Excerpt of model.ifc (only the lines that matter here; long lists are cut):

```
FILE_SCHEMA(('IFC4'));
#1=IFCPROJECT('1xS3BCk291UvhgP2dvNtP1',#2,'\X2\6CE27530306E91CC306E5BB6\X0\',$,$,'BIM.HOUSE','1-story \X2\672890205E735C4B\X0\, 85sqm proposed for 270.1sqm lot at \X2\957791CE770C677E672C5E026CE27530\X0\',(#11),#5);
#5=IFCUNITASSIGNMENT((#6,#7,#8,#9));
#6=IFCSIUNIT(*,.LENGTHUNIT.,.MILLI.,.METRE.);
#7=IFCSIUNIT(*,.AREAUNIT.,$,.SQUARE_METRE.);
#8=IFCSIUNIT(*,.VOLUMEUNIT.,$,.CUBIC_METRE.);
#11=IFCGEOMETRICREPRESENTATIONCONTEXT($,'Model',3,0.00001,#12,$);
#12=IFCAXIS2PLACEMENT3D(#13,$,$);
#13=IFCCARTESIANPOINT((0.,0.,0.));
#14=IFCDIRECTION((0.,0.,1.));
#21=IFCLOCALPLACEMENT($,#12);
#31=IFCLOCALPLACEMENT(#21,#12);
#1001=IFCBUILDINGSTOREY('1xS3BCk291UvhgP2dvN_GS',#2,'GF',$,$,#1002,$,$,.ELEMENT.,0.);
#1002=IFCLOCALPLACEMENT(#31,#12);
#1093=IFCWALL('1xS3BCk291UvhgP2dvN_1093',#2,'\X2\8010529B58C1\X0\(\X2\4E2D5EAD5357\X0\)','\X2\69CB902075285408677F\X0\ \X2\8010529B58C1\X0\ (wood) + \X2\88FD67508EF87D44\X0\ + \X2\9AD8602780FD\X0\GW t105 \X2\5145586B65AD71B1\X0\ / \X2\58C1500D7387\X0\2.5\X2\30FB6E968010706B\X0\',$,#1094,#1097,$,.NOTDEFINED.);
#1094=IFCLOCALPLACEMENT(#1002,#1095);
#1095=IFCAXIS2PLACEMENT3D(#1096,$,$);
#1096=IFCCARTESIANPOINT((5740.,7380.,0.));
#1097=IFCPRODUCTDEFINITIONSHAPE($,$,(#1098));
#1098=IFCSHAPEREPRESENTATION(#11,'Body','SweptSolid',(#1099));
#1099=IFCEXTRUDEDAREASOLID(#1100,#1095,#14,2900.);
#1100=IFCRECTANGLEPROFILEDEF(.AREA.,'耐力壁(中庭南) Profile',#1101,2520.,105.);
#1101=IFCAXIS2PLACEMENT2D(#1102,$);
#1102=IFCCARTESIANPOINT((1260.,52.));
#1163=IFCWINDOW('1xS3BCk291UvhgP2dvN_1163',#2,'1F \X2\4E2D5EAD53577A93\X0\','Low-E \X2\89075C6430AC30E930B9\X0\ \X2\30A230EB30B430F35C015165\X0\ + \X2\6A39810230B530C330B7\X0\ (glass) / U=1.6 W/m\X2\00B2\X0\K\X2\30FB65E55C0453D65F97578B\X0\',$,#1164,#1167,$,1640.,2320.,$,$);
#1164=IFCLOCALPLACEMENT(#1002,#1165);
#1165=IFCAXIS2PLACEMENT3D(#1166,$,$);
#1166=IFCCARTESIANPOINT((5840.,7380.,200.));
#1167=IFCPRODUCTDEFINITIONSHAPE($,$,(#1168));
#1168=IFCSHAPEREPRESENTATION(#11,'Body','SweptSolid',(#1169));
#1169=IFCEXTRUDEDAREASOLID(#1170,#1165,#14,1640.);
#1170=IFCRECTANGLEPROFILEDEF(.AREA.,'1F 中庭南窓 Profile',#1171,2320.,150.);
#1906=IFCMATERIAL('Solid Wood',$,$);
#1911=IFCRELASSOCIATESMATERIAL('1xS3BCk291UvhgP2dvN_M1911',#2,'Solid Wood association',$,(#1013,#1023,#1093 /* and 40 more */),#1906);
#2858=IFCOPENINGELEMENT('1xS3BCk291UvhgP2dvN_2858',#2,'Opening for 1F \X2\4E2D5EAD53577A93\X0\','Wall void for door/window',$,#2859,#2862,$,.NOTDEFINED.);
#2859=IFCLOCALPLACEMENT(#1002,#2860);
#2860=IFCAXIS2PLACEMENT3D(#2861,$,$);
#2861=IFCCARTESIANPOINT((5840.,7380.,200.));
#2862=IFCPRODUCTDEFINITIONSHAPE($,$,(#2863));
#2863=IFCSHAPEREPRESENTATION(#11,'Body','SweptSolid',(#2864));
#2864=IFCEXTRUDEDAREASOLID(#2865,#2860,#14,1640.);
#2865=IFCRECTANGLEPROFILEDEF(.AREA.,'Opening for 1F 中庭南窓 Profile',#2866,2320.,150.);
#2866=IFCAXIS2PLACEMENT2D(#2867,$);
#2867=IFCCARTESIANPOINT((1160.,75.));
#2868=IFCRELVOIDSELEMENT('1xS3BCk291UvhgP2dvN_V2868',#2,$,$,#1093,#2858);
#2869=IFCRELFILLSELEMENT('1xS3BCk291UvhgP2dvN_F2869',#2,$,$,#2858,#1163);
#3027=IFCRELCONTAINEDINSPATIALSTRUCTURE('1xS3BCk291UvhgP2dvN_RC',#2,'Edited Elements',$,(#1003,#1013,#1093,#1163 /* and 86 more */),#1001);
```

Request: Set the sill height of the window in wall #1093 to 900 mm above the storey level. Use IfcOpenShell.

```python
import numpy as np
import ifcopenshell
import ifcopenshell.api.geometry
import ifcopenshell.geom
import ifcopenshell.util.element
import ifcopenshell.util.placement
import ifcopenshell.util.shape
import ifcopenshell.util.unit

model = ifcopenshell.open("model.ifc")
unit_scale = ifcopenshell.util.unit.calculate_unit_scale(model)

window = model.by_guid("1xS3BCk291UvhgP2dvN_1163")
opening = window.FillsVoids[0].RelatingOpeningElement
storey = ifcopenshell.util.element.get_container(window, ifc_class="IfcBuildingStorey")
level = ifcopenshell.util.placement.get_local_placement(storey.ObjectPlacement)[2, 3]

# The opening's origin need not be at the sill, so measure its lowest point.
shape = ifcopenshell.geom.create_shape(ifcopenshell.geom.settings(), opening)
bottom = ifcopenshell.util.shape.get_shape_bottom_elevation(shape, shape.geometry) / unit_scale
dz = level + 0.9 / unit_scale - bottom

shift = np.array([0.0, 0.0, dz])
# The window is not placed relative to its opening, so move both.
for product in (opening, window):
    matrix = ifcopenshell.util.placement.get_local_placement(product.ObjectPlacement)
    matrix[:3, 3] += shift
    ifcopenshell.api.geometry.edit_object_placement(model, product=product, matrix=matrix, is_si=False)

print(f"moved by {dz * unit_scale:+.3f} m")

model.write("model_v2.ifc")
```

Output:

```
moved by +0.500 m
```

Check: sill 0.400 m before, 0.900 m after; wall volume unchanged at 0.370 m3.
